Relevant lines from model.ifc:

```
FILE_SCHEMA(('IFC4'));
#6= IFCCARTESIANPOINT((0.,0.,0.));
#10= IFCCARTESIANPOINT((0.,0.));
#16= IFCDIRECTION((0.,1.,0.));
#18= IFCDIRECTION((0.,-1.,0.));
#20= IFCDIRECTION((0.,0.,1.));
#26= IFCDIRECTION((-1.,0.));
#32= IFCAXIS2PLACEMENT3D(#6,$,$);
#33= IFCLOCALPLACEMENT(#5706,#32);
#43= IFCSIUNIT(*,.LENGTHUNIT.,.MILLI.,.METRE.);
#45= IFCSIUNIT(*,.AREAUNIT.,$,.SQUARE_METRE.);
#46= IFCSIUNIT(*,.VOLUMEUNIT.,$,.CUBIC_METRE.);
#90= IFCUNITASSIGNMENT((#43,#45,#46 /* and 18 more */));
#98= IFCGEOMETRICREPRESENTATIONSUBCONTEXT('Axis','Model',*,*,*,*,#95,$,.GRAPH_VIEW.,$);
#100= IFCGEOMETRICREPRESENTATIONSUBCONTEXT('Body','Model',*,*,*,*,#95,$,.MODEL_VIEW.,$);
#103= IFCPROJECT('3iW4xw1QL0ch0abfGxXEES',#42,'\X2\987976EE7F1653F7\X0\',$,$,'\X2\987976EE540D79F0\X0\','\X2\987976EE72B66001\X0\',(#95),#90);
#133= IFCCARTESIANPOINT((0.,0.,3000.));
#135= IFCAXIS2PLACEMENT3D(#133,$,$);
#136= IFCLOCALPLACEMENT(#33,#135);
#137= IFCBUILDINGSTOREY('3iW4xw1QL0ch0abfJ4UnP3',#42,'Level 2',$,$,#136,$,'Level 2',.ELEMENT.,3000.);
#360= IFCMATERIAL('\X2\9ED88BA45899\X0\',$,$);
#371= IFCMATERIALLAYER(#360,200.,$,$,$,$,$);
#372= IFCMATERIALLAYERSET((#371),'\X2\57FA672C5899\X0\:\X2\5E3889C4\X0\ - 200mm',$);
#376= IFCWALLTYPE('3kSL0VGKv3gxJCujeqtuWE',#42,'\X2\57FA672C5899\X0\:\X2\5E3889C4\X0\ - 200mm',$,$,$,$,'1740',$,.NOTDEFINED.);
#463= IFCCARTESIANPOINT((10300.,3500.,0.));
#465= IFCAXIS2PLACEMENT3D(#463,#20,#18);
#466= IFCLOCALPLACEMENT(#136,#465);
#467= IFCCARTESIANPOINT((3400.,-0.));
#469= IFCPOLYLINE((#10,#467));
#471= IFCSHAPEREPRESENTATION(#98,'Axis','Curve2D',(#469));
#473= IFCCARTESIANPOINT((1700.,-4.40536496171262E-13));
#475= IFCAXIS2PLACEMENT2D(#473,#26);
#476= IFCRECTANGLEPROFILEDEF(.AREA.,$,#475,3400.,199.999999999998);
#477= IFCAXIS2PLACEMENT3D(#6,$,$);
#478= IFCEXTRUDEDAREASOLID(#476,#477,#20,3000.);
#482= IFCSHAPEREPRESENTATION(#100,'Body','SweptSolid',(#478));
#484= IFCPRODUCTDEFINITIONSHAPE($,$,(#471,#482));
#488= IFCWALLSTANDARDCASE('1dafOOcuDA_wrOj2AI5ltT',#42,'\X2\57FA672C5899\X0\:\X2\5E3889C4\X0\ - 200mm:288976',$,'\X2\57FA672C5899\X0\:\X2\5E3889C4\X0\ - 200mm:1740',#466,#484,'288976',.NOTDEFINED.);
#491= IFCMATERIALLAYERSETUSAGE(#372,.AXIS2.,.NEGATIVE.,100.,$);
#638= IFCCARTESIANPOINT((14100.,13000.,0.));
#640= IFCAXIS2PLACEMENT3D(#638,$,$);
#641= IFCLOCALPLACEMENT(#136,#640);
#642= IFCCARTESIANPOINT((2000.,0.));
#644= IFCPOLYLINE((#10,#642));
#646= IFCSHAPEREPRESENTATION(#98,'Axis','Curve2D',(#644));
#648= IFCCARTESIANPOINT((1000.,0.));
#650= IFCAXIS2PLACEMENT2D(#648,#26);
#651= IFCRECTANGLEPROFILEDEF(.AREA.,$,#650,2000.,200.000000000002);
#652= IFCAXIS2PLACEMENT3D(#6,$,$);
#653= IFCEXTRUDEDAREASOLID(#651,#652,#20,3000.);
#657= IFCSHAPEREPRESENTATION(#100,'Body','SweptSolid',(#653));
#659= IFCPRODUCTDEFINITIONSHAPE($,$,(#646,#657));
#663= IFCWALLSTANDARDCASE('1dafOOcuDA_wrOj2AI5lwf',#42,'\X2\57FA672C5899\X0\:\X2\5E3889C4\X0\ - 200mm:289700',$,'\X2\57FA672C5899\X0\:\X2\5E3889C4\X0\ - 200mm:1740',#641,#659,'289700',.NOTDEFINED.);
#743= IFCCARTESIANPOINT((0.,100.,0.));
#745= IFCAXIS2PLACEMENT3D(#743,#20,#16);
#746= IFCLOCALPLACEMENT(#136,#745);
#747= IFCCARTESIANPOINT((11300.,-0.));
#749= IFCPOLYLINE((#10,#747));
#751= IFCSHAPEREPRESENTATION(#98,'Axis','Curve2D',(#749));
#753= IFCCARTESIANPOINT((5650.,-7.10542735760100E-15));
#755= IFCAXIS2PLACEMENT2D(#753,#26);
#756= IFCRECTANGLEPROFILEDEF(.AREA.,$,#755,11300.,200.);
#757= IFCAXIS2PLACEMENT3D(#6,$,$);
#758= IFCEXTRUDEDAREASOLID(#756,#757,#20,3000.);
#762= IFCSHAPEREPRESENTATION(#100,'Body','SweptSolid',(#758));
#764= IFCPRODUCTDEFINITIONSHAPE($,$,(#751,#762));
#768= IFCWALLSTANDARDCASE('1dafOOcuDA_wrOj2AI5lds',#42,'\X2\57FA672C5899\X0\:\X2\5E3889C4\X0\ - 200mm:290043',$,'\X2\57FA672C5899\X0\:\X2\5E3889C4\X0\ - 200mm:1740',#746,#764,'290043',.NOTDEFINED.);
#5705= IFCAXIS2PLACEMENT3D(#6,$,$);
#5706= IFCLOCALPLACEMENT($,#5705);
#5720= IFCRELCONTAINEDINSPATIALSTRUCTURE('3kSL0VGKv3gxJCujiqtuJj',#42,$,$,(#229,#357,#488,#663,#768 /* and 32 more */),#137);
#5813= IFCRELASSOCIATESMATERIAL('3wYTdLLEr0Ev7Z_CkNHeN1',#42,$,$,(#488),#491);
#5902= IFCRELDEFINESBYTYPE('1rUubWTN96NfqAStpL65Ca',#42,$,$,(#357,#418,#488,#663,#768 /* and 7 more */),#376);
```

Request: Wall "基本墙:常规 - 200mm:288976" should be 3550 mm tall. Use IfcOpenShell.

```python
import ifcopenshell
import ifcopenshell.geom
import ifcopenshell.util.representation
import ifcopenshell.util.shape
import ifcopenshell.util.unit

model = ifcopenshell.open("model.ifc")
unit_scale = ifcopenshell.util.unit.calculate_unit_scale(model)
settings = ifcopenshell.geom.settings()


def volume(element):
    """Net volume in cubic metres, openings subtracted."""
    shape = ifcopenshell.geom.create_shape(settings, element)
    return ifcopenshell.util.shape.get_volume(shape.geometry)


wall = model.by_id(488)
before = volume(wall)

body = ifcopenshell.util.representation.get_representation(wall, "Model", "Body")
solid = body.Items[0]
old_height = solid.Depth
solid.Depth = 3.55 / unit_scale
after = volume(wall)

print(f"height {old_height:g} -> {solid.Depth:g}, volume {before:.3f} -> {after:.3f} m3")

model.write("model_rev.ifc")
```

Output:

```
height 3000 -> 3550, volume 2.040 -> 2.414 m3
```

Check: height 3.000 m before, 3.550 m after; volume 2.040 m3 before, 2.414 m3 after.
